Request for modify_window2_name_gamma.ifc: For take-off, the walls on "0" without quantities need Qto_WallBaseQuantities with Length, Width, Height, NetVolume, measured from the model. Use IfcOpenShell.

First a look at what the model holds.

```python
import ifcopenshell
import ifcopenshell.util.element
import ifcopenshell.util.unit

model = ifcopenshell.open("modify_window2_name_gamma.ifc")
print(model.schema)
for unit_type in ("LENGTHUNIT", "AREAUNIT", "VOLUMEUNIT"):
    print(unit_type, ifcopenshell.util.unit.calculate_unit_scale(model, unit_type))
storey = next(s for s in model.by_type("IfcBuildingStorey") if s.Name == "0")
walls = [e for e in ifcopenshell.util.element.get_decomposition(storey) if e.is_a("IfcWall")]
for e in sorted(walls, key=lambda e: e.id()):
    print(e.id(), e.is_a(), e.Name, list(ifcopenshell.util.element.get_psets(e, qtos_only=True)), sep=" | ")
```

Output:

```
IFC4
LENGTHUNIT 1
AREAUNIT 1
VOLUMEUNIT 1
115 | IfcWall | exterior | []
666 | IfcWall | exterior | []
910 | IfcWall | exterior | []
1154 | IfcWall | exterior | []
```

```python
import ifcopenshell
import ifcopenshell.api.pset
import ifcopenshell.geom
import ifcopenshell.util.element
import ifcopenshell.util.shape
import ifcopenshell.util.unit

model = ifcopenshell.open("modify_window2_name_gamma.ifc")
unit_scale = ifcopenshell.util.unit.calculate_unit_scale(model)
volume_scale = ifcopenshell.util.unit.calculate_unit_scale(model, "VOLUMEUNIT")
settings = ifcopenshell.geom.settings()

storey = next(s for s in model.by_type("IfcBuildingStorey") if s.Name == "0")
walls = [e for e in ifcopenshell.util.element.get_decomposition(storey) if e.is_a("IfcWall")]

for e in sorted(walls, key=lambda e: e.id()):
    if ifcopenshell.util.element.get_psets(e, qtos_only=True, should_inherit=False):
        continue
    # Geometry comes back in metres, in the element's own axes.
    shape = ifcopenshell.geom.create_shape(settings, e)
    values = {
        "Length": ifcopenshell.util.shape.get_x(shape.geometry) / unit_scale,
        "Width": ifcopenshell.util.shape.get_y(shape.geometry) / unit_scale,
        "Height": ifcopenshell.util.shape.get_z(shape.geometry) / unit_scale,
        "NetVolume": ifcopenshell.util.shape.get_volume(shape.geometry) / volume_scale,
    }
    qto = ifcopenshell.api.pset.add_qto(model, product=e, name="Qto_WallBaseQuantities")
    ifcopenshell.api.pset.edit_qto(model, qto=qto, properties=values)
    print(e.id(), {k: round(v, 3) for k, v in values.items()})

model.write("modify_window2_name_gamma-out.ifc")
```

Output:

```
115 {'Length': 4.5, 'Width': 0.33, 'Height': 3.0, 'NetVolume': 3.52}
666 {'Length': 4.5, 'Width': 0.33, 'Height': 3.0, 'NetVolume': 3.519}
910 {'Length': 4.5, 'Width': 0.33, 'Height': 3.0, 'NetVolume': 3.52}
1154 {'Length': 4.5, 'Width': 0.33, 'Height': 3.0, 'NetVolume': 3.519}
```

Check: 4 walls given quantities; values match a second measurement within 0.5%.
